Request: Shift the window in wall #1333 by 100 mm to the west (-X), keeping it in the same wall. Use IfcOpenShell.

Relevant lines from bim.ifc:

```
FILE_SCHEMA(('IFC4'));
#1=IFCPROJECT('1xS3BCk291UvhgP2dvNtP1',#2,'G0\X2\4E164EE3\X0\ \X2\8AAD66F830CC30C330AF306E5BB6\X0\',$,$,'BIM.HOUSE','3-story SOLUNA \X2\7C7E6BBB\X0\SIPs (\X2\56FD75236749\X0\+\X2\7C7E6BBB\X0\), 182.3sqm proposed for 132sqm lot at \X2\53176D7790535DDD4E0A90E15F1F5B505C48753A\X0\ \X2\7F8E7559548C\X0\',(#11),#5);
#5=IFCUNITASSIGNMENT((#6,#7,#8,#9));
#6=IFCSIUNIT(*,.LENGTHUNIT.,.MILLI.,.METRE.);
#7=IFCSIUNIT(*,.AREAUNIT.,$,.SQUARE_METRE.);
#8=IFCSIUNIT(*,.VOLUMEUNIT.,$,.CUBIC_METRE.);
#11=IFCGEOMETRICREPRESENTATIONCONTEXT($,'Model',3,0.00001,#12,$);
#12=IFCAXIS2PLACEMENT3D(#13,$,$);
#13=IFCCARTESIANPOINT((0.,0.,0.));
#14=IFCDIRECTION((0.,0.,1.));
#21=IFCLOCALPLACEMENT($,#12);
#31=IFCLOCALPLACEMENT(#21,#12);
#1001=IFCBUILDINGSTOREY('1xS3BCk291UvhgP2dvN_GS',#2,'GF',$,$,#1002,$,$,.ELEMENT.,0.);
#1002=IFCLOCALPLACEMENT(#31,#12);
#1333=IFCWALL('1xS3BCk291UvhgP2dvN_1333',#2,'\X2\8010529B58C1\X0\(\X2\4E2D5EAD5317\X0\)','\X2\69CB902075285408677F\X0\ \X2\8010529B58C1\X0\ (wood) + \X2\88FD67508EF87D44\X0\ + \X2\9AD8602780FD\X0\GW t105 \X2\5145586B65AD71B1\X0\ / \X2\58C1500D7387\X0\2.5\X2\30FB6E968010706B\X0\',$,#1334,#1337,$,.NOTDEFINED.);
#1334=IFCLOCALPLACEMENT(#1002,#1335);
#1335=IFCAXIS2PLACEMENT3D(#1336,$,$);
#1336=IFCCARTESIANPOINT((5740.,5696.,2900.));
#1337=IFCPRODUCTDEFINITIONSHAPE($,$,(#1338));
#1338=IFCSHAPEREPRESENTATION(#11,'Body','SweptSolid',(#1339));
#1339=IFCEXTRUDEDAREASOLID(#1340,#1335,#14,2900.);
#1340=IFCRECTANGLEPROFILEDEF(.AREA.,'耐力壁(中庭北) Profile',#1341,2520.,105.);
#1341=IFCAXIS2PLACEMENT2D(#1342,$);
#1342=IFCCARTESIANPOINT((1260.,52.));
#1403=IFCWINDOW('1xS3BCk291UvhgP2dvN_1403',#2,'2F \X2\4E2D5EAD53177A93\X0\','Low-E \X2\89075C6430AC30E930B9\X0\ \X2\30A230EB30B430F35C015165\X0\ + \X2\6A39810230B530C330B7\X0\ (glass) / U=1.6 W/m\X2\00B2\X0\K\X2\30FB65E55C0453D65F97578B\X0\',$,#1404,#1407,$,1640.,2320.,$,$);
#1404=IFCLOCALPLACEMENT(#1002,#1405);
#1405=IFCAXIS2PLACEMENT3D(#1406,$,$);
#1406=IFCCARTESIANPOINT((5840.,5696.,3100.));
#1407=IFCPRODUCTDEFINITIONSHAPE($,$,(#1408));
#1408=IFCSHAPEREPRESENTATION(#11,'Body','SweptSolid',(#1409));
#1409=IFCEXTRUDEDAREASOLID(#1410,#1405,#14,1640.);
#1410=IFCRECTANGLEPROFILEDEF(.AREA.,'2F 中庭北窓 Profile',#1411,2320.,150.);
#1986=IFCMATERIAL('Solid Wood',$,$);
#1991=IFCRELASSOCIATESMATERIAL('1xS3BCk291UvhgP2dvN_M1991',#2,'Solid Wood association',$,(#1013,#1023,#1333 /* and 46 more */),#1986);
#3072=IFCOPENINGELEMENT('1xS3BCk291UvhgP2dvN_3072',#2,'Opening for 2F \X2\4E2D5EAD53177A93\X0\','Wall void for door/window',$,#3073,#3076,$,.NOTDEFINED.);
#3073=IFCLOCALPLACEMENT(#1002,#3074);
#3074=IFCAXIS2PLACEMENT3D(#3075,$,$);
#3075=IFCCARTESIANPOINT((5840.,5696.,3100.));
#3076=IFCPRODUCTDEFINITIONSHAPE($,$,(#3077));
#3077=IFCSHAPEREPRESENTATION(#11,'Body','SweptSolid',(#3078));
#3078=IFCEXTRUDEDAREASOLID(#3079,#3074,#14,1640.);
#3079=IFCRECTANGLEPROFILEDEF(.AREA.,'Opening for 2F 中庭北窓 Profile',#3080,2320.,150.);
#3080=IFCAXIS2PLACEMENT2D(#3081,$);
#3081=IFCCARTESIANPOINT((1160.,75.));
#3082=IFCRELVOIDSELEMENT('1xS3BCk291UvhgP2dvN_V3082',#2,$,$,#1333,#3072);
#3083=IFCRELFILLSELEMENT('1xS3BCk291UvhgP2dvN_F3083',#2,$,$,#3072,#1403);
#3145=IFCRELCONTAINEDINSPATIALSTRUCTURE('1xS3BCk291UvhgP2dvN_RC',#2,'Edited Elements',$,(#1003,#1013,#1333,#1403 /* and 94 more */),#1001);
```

```python
import ifcopenshell
import ifcopenshell.api.geometry
import ifcopenshell.util.placement
import ifcopenshell.util.unit

model = ifcopenshell.open("bim.ifc")
unit_scale = ifcopenshell.util.unit.calculate_unit_scale(model)

window = model.by_guid("1xS3BCk291UvhgP2dvN_1403")
opening = window.FillsVoids[0].RelatingOpeningElement
wall = opening.VoidsElements[0].RelatingBuildingElement

wall_matrix = ifcopenshell.util.placement.get_local_placement(wall.ObjectPlacement)
shift = wall_matrix[:3, 0] * -0.1 / unit_scale
before = ifcopenshell.util.placement.get_local_placement(window.ObjectPlacement)[:3, 3].copy()

# The window is not placed relative to its opening, so move both.
for product in (opening, window):
    matrix = ifcopenshell.util.placement.get_local_placement(product.ObjectPlacement)
    matrix[:3, 3] += shift
    ifcopenshell.api.geometry.edit_object_placement(model, product=product, matrix=matrix, is_si=False)

after = ifcopenshell.util.placement.get_local_placement(window.ObjectPlacement)[:3, 3]
print("window moved by", (after - before).round(3) + 0.0)

model.write("bim_v2.ifc")
```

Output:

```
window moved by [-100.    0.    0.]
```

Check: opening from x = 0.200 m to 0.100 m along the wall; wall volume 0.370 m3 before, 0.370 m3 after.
